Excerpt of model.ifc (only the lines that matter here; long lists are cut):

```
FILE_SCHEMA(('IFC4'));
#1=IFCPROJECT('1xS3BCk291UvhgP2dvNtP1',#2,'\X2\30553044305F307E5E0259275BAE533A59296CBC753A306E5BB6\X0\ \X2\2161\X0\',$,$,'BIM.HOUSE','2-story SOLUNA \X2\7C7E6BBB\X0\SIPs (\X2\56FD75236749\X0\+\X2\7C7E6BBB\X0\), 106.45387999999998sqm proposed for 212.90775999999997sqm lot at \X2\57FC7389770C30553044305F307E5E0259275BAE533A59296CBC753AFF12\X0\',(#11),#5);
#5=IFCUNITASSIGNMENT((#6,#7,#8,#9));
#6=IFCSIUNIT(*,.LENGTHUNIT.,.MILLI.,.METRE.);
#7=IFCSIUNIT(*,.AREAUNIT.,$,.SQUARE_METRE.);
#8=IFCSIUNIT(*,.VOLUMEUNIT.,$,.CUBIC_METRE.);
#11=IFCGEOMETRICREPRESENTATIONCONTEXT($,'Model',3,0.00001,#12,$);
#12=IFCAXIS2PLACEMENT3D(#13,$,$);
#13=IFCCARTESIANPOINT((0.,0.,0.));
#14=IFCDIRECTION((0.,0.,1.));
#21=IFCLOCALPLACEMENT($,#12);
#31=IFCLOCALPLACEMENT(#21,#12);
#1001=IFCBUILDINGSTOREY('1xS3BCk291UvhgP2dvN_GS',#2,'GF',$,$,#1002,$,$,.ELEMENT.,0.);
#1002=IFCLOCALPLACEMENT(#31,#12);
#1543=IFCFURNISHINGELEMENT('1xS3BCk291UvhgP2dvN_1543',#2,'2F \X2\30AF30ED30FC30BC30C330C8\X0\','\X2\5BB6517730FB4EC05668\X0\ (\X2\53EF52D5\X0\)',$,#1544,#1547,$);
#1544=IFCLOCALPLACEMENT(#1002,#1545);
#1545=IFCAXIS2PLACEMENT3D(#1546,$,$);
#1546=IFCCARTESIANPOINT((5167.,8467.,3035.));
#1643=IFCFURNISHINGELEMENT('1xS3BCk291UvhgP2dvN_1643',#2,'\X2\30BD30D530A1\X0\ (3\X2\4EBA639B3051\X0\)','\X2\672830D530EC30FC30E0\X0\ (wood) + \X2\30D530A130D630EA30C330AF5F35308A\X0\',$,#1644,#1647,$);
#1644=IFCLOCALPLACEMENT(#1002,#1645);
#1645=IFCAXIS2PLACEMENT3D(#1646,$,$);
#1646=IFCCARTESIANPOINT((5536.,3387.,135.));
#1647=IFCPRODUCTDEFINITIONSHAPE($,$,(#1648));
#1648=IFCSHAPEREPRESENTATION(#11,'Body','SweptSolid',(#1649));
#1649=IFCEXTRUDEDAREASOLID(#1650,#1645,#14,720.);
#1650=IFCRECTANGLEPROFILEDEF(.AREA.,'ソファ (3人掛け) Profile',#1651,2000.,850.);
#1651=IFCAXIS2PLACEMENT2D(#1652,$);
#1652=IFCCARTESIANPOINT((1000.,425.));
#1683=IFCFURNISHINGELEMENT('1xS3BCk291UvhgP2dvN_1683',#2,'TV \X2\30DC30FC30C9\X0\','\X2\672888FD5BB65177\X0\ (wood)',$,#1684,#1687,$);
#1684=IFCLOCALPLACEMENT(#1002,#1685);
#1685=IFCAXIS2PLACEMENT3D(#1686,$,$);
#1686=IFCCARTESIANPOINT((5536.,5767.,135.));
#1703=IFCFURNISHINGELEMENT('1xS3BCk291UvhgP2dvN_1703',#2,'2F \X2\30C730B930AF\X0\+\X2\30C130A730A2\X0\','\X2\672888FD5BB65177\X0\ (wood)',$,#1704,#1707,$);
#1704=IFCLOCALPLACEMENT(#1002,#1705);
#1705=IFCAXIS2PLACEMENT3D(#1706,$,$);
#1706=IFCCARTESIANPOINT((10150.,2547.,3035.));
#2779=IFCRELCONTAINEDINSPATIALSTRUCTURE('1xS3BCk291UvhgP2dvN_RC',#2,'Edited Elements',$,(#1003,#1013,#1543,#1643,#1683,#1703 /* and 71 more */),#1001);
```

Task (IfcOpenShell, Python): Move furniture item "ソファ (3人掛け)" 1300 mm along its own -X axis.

```python
import ifcopenshell
import ifcopenshell.api.geometry
import ifcopenshell.util.placement
import ifcopenshell.util.unit

model = ifcopenshell.open("model.ifc")
unit_scale = ifcopenshell.util.unit.calculate_unit_scale(model)

item = model.by_guid("1xS3BCk291UvhgP2dvN_1643")
matrix = ifcopenshell.util.placement.get_local_placement(item.ObjectPlacement)
matrix[:3, 3] -= matrix[:3, 0] * 1.3 / unit_scale
ifcopenshell.api.geometry.edit_object_placement(model, product=item, matrix=matrix, is_si=False)

print(ifcopenshell.util.placement.get_local_placement(item.ObjectPlacement).round(3) + 0.0)

model.write("model-out.ifc")
```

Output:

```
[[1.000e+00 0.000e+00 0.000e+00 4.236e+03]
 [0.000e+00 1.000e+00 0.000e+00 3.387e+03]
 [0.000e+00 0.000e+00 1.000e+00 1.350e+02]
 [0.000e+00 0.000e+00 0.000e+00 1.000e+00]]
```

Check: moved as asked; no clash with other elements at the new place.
